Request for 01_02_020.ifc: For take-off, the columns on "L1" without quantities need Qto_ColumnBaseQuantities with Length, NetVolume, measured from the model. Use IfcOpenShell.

First a look at what the model holds.

```python
import ifcopenshell
import ifcopenshell.util.element
import ifcopenshell.util.unit

model = ifcopenshell.open("01_02_020.ifc")
print(model.schema)
for unit_type in ("LENGTHUNIT", "AREAUNIT", "VOLUMEUNIT"):
    print(unit_type, ifcopenshell.util.unit.calculate_unit_scale(model, unit_type))
storey = next(s for s in model.by_type("IfcBuildingStorey") if s.Name == "L1")
columns = [e for e in ifcopenshell.util.element.get_decomposition(storey) if e.is_a("IfcColumn")]
for e in sorted(columns, key=lambda e: e.id()):
    print(e.id(), e.is_a(), e.Name, list(ifcopenshell.util.element.get_psets(e, qtos_only=True)), sep=" | ")
```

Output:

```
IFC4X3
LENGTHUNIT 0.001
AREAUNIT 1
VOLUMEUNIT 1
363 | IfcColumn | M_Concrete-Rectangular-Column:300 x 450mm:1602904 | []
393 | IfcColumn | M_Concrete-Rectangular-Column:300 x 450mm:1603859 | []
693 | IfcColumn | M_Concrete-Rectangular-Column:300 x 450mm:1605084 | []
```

```python
import ifcopenshell
import ifcopenshell.api.pset
import ifcopenshell.geom
import ifcopenshell.util.element
import ifcopenshell.util.shape
import ifcopenshell.util.unit

model = ifcopenshell.open("01_02_020.ifc")
unit_scale = ifcopenshell.util.unit.calculate_unit_scale(model)
volume_scale = ifcopenshell.util.unit.calculate_unit_scale(model, "VOLUMEUNIT")
settings = ifcopenshell.geom.settings()

storey = next(s for s in model.by_type("IfcBuildingStorey") if s.Name == "L1")
columns = [e for e in ifcopenshell.util.element.get_decomposition(storey) if e.is_a("IfcColumn")]

for e in sorted(columns, key=lambda e: e.id()):
    if ifcopenshell.util.element.get_psets(e, qtos_only=True, should_inherit=False):
        continue
    # Geometry comes back in metres, in the element's own axes.
    shape = ifcopenshell.geom.create_shape(settings, e)
    values = {
        "Length": ifcopenshell.util.shape.get_z(shape.geometry) / unit_scale,
        "NetVolume": ifcopenshell.util.shape.get_volume(shape.geometry) / volume_scale,
    }
    qto = ifcopenshell.api.pset.add_qto(model, product=e, name="Qto_ColumnBaseQuantities")
    ifcopenshell.api.pset.edit_qto(model, qto=qto, properties=values)
    print(e.id(), {k: round(v, 3) for k, v in values.items()})

model.write("01_02_020_v2.ifc")
```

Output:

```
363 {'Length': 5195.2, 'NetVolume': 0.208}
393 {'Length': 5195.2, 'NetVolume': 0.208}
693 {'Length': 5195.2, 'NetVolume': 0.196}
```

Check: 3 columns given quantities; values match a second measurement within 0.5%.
